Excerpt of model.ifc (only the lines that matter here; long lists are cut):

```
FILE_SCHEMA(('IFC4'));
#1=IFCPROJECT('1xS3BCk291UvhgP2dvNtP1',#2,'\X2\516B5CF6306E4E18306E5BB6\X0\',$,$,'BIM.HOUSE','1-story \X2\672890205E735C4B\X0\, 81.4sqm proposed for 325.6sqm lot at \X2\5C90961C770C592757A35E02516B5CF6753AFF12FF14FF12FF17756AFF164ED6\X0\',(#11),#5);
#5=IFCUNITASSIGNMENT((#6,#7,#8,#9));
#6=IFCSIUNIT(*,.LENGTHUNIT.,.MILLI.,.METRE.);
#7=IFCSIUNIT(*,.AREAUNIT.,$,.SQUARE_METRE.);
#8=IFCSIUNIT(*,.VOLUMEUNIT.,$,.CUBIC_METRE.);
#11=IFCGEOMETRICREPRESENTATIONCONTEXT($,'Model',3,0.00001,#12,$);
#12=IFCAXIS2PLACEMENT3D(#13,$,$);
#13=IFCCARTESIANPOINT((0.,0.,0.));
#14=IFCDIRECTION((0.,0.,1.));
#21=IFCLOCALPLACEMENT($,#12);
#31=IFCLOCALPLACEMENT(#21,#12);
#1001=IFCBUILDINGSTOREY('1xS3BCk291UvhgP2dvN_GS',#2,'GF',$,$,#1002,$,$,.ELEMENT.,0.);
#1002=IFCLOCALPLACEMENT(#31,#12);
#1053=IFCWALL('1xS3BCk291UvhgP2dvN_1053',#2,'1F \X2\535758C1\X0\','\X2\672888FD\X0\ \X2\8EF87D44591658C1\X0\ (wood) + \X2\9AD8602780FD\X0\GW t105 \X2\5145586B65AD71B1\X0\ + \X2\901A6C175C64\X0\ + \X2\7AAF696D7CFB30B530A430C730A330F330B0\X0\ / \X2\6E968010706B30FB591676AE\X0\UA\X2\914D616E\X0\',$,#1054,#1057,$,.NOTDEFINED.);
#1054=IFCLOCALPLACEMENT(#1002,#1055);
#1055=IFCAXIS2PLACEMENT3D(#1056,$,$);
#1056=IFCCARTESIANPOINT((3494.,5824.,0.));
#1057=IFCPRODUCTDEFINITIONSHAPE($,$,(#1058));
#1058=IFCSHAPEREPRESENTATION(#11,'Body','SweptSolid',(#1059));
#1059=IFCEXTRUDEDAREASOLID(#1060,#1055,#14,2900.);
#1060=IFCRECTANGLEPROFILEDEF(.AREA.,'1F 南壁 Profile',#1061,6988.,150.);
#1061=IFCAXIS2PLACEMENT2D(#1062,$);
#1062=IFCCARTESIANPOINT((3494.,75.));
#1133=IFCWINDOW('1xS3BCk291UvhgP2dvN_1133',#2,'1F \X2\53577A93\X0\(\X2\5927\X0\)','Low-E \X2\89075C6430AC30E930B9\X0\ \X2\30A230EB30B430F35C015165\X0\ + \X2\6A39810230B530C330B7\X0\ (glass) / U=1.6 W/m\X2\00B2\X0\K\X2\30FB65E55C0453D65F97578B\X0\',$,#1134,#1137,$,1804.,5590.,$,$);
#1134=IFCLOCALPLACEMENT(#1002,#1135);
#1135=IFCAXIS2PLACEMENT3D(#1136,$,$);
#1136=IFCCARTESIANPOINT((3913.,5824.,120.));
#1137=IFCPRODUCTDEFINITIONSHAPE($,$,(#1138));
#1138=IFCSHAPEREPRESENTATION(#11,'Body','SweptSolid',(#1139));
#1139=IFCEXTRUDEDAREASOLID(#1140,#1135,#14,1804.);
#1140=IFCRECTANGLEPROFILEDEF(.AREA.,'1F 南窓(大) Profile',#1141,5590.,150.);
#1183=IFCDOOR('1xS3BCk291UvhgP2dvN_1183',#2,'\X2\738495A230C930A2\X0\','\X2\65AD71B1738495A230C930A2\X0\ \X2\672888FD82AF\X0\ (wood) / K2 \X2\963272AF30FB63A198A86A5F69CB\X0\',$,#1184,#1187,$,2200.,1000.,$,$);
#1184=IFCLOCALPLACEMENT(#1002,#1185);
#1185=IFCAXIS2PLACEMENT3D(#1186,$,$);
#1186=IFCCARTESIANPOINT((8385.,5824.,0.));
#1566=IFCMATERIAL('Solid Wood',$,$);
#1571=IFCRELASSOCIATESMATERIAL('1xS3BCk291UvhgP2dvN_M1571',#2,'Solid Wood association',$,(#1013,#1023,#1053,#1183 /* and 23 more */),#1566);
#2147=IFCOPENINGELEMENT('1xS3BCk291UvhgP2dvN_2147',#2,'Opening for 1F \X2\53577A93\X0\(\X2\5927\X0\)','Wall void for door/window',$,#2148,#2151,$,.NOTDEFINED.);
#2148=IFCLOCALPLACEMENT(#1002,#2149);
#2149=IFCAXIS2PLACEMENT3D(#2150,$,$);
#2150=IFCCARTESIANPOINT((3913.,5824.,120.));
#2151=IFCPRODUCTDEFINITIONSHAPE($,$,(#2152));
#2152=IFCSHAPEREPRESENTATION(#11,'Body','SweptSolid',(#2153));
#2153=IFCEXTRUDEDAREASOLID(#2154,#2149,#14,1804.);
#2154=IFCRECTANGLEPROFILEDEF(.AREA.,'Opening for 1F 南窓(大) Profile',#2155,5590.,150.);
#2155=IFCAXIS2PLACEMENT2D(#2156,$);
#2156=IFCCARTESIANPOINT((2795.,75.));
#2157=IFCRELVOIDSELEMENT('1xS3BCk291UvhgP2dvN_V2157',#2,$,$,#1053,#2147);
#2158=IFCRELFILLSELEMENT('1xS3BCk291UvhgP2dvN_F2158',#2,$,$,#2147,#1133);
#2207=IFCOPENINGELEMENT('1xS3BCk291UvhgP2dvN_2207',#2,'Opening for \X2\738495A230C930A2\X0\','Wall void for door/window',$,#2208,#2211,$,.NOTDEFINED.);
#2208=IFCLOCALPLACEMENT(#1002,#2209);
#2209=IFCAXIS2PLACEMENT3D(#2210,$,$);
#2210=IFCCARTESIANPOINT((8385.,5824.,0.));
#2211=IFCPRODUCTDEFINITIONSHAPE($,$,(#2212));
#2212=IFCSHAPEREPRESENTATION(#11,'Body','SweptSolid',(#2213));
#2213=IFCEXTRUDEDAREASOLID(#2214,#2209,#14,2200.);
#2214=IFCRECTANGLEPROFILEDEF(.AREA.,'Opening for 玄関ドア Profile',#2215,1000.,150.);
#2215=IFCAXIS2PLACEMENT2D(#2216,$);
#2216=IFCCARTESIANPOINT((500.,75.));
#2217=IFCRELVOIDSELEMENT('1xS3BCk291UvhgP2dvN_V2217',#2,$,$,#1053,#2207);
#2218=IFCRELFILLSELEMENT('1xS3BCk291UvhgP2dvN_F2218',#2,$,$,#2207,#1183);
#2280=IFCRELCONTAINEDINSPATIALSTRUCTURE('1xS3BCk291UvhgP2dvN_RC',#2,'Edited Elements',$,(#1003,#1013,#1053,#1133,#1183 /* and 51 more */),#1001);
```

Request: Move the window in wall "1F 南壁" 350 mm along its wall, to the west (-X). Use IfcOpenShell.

```python
import ifcopenshell
import ifcopenshell.api.geometry
import ifcopenshell.util.placement

model = ifcopenshell.open("model.ifc")

window = model.by_id(1133)
opening = window.FillsVoids[0].RelatingOpeningElement
wall = opening.VoidsElements[0].RelatingBuildingElement

wall_matrix = ifcopenshell.util.placement.get_local_placement(wall.ObjectPlacement)
shift = wall_matrix[:3, 0] * -350.0
before = ifcopenshell.util.placement.get_local_placement(window.ObjectPlacement)[:3, 3].copy()

# The window is not placed relative to its opening, so move both.
for product in (opening, window):
    matrix = ifcopenshell.util.placement.get_local_placement(product.ObjectPlacement)
    matrix[:3, 3] += shift
    ifcopenshell.api.geometry.edit_object_placement(model, product=product, matrix=matrix, is_si=False)

after = ifcopenshell.util.placement.get_local_placement(window.ObjectPlacement)[:3, 3]
print("window moved by", (after - before).round(3) + 0.0)

model.write("model_rev.ifc")
```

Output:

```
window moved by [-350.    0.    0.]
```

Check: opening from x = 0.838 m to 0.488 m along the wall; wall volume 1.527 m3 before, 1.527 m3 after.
